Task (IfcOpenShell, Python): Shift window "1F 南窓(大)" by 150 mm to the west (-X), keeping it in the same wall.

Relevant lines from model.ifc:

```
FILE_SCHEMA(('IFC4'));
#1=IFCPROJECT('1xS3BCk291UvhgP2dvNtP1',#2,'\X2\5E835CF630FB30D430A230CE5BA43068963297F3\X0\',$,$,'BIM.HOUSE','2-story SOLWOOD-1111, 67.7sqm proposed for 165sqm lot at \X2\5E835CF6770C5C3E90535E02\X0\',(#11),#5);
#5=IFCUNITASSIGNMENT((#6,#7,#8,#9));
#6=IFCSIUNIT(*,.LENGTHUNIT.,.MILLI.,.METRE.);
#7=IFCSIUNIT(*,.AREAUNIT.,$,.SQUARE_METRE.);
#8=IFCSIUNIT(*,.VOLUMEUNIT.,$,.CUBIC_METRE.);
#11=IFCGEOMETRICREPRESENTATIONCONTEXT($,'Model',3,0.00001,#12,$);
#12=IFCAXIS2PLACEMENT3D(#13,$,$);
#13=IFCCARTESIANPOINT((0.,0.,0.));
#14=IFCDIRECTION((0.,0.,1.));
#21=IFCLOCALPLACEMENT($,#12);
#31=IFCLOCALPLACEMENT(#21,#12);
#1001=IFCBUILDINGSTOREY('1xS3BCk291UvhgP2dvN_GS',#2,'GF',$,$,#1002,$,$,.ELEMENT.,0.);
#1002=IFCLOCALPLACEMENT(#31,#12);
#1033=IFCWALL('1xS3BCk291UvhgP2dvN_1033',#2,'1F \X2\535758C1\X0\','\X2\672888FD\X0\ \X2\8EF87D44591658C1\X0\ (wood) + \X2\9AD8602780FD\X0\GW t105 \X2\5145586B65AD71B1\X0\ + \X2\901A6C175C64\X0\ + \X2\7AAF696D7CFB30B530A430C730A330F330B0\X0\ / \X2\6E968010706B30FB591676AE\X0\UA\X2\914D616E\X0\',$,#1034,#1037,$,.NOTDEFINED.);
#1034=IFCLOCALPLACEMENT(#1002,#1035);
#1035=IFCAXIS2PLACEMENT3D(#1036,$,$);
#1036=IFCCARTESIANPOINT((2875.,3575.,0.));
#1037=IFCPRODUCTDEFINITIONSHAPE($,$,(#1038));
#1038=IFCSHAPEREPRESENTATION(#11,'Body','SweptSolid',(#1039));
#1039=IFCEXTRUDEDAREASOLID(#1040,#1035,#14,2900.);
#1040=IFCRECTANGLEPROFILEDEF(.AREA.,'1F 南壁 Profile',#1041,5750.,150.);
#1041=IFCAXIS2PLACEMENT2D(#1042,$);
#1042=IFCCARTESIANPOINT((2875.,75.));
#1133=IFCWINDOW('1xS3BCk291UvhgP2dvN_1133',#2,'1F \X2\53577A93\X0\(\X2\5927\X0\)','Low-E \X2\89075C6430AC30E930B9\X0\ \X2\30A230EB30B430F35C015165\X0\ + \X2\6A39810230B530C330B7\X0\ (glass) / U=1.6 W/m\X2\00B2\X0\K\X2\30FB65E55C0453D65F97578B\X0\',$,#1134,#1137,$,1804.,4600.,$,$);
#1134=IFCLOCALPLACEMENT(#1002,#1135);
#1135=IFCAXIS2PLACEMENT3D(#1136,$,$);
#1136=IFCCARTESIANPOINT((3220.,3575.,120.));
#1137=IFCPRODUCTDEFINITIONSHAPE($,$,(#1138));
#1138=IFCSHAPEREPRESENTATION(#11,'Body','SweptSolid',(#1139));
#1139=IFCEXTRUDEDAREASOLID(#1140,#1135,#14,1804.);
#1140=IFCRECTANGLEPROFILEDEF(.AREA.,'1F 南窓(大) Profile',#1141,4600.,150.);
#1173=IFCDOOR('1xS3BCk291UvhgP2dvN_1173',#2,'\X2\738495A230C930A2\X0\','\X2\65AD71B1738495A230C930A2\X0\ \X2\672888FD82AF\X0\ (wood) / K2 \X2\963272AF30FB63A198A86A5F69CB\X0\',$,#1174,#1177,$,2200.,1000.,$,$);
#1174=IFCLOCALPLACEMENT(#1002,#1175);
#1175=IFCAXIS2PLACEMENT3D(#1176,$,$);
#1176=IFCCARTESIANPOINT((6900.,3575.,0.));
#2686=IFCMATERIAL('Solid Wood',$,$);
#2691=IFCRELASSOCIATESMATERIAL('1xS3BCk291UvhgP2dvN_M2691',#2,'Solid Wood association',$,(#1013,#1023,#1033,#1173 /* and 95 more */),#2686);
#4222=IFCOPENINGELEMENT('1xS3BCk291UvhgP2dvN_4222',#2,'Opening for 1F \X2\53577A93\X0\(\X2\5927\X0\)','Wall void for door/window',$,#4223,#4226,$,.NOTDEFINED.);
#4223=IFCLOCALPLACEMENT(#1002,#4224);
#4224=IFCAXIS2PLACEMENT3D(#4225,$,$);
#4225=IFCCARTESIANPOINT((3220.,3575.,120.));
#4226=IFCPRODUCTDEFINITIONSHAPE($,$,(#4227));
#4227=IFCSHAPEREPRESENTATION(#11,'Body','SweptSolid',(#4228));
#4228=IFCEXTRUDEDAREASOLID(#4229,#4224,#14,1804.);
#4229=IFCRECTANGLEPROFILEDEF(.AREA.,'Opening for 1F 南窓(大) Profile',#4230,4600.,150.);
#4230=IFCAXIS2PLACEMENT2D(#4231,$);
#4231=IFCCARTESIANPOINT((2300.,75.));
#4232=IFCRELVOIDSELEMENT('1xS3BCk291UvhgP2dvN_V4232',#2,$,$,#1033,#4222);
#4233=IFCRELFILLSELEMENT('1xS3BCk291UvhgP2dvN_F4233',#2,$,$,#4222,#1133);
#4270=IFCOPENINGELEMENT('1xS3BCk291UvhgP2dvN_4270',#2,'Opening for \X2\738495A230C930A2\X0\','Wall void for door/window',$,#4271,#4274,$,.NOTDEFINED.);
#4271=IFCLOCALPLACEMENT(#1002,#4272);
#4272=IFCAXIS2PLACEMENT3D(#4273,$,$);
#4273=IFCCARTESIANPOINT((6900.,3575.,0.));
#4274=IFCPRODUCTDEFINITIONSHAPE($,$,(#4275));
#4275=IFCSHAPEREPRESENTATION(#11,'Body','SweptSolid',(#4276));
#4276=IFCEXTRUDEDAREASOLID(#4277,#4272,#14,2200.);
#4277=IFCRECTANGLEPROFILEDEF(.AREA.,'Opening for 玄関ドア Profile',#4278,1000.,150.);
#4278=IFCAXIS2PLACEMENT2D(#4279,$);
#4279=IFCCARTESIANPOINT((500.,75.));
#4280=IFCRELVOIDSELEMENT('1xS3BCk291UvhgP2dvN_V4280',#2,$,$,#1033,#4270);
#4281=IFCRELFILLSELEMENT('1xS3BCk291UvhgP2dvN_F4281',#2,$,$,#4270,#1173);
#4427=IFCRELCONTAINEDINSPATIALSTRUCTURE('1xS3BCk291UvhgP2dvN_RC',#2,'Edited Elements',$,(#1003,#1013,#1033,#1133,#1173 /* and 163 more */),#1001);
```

```python
import ifcopenshell
import ifcopenshell.api.geometry
import ifcopenshell.util.placement

model = ifcopenshell.open("model.ifc")

window = model.by_guid("1xS3BCk291UvhgP2dvN_1133")
opening = window.FillsVoids[0].RelatingOpeningElement
wall = opening.VoidsElements[0].RelatingBuildingElement

wall_matrix = ifcopenshell.util.placement.get_local_placement(wall.ObjectPlacement)
shift = wall_matrix[:3, 0] * -150.0
before = ifcopenshell.util.placement.get_local_placement(window.ObjectPlacement)[:3, 3].copy()

# The window is not placed relative to its opening, so move both.
for product in (opening, window):
    matrix = ifcopenshell.util.placement.get_local_placement(product.ObjectPlacement)
    matrix[:3, 3] += shift
    ifcopenshell.api.geometry.edit_object_placement(model, product=product, matrix=matrix, is_si=False)

after = ifcopenshell.util.placement.get_local_placement(window.ObjectPlacement)[:3, 3]
print("window moved by", (after - before).round(3) + 0.0)

model.write("model_v2.ifc")
```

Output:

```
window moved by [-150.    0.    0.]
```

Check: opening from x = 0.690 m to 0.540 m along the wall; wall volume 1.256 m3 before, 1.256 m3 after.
